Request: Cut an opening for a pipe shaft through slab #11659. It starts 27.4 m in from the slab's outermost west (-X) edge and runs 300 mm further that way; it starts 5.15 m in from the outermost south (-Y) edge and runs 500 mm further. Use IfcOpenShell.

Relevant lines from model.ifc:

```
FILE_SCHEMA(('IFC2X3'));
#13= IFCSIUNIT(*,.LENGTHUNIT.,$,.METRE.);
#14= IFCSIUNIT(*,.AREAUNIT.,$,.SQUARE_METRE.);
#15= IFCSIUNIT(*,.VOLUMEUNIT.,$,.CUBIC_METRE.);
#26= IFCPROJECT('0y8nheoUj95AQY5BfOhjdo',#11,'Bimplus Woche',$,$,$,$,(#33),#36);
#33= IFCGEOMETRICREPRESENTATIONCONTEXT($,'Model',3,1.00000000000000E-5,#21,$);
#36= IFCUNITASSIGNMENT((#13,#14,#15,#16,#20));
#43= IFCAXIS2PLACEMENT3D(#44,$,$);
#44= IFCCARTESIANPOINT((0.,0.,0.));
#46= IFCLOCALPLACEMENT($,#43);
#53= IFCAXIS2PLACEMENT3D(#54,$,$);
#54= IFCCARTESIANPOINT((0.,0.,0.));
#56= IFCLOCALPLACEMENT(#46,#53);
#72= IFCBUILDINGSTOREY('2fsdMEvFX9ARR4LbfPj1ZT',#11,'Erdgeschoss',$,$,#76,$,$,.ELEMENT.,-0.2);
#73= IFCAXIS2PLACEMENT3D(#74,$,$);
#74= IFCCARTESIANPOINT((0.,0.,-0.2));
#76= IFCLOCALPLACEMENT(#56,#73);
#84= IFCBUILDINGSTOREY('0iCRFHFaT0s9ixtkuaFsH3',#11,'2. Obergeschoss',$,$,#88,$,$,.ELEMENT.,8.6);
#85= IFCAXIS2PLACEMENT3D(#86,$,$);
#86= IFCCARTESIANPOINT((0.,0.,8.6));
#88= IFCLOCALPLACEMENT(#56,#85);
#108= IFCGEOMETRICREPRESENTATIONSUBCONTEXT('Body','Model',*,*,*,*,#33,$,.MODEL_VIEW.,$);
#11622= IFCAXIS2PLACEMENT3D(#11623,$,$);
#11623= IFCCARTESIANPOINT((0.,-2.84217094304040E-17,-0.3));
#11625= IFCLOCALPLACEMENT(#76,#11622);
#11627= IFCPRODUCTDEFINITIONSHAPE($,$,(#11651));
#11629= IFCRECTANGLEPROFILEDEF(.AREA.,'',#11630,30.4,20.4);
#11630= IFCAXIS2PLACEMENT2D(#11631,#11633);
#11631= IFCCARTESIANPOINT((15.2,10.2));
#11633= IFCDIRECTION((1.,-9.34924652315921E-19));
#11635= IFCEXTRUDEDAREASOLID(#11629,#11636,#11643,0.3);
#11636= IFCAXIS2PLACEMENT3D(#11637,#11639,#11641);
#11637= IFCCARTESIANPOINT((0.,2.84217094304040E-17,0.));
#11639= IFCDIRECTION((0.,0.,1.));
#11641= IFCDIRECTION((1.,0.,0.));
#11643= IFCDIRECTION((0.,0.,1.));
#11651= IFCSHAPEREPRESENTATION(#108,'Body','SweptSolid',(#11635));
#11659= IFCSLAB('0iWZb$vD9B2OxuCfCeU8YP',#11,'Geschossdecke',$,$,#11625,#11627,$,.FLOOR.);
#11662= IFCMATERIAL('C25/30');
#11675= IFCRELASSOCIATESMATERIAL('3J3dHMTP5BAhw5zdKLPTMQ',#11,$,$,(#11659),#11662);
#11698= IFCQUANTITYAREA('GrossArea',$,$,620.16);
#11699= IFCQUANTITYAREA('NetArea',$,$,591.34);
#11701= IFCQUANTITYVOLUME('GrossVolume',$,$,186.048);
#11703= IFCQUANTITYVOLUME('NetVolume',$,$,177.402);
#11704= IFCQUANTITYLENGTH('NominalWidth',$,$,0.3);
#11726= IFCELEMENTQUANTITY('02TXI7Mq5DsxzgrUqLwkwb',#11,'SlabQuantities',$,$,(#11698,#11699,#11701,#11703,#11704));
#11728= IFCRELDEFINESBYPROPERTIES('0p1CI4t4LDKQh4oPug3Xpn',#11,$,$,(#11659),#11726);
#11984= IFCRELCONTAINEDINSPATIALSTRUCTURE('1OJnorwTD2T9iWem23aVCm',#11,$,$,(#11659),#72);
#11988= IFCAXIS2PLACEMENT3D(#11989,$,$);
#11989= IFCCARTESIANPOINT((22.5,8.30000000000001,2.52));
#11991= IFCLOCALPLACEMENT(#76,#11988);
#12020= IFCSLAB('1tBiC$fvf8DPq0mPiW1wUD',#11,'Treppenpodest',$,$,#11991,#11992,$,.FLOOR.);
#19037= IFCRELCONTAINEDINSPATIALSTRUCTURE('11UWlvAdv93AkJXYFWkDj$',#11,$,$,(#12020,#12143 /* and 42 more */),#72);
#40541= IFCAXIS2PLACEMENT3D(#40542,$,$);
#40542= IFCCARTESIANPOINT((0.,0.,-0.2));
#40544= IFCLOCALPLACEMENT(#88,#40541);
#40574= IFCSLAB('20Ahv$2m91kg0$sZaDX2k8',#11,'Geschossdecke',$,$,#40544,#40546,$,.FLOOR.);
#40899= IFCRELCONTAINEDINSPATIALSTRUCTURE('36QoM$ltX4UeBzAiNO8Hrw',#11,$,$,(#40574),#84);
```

```python
import numpy as np
import ifcopenshell
import ifcopenshell.api.feature
import ifcopenshell.api.geometry
import ifcopenshell.api.pset
import ifcopenshell.api.root
import ifcopenshell.geom
import ifcopenshell.util.element
import ifcopenshell.util.placement
import ifcopenshell.util.representation
import ifcopenshell.util.shape
import ifcopenshell.util.unit

model = ifcopenshell.open("model.ifc")
unit_scale = ifcopenshell.util.unit.calculate_unit_scale(model)
area_scale = ifcopenshell.util.unit.calculate_unit_scale(model, "AREAUNIT")
volume_scale = ifcopenshell.util.unit.calculate_unit_scale(model, "VOLUMEUNIT")
settings = ifcopenshell.geom.settings()


def volume(element):
    """Net volume in cubic metres, openings subtracted."""
    shape = ifcopenshell.geom.create_shape(settings, element)
    return ifcopenshell.util.shape.get_volume(shape.geometry)


slab = model.by_guid("0iWZb$vD9B2OxuCfCeU8YP")
before = volume(slab)

# Extent in the slab's own axes, in metres. The edges named are its -X and -Y sides.
slab_shape = ifcopenshell.geom.create_shape(settings, slab)
vertices = ifcopenshell.util.shape.get_vertices(slab_shape.geometry)
x_min, y_min, bottom = vertices.min(axis=0)
top = vertices[:, 2].max()

opening = ifcopenshell.api.root.create_entity(model, ifc_class="IfcOpeningElement", name="Pipe shaft opening")
context = ifcopenshell.util.representation.get_context(model, "Model", "Body", "MODEL_VIEW")
width, depth = 0.3, 0.5
outline = [(0.0, 0.0), (width, 0.0), (width, depth), (0.0, depth), (0.0, 0.0)]
# Overshoot both faces by 50 mm so the cut is clean.
shape = ifcopenshell.api.geometry.add_slab_representation(
    model, context=context, depth=top - bottom + 0.1, polyline=outline
)
ifcopenshell.api.geometry.assign_representation(model, product=opening, representation=shape)

matrix = ifcopenshell.util.placement.get_local_placement(slab.ObjectPlacement)
matrix[:, 3] = matrix @ np.append(np.array([x_min + 27.4, y_min + 5.15, bottom - 0.05]) / unit_scale, 1.0)
ifcopenshell.api.geometry.edit_object_placement(model, product=opening, matrix=matrix, is_si=False)
ifcopenshell.api.feature.add_feature(model, feature=opening, element=slab)

after = volume(slab)

# Update the slab's stored quantities.
qto = model.by_id(ifcopenshell.util.element.get_pset(slab, "SlabQuantities", should_inherit=False)["id"])
ifcopenshell.api.pset.edit_qto(model, qto=qto, properties={
    "NetArea": after / (top - bottom) / area_scale,
    "NetVolume": after / volume_scale,
})

print(f"slab volume {before:.3f} -> {after:.3f} m3")

model.write("model-out.ifc")
```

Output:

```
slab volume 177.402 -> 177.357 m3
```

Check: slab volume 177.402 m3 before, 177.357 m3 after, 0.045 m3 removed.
